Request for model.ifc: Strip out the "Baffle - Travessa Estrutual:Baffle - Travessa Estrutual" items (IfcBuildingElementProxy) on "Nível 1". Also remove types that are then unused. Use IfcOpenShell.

First a look at what the model holds.

```python
import ifcopenshell
import ifcopenshell.util.element

model = ifcopenshell.open("model.ifc")
print(model.schema)
storey = next(s for s in model.by_type("IfcBuildingStorey") if s.Name == "Nível 1")
proxies = [e for e in ifcopenshell.util.element.get_decomposition(storey) if e.is_a("IfcBuildingElementProxy")]
seen = {}
for e in proxies:
    element_type = ifcopenshell.util.element.get_type(e)
    name = element_type.Name if element_type not in (None, e) else None
    seen[name] = seen.get(name, 0) + 1
for name, count in sorted(seen.items(), key=str):
    print(count, "x", name)
```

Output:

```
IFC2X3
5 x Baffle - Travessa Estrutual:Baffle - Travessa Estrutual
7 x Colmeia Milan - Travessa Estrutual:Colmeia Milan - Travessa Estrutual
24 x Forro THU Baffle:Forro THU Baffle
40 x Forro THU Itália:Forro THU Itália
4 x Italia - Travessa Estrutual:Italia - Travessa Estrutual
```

```python
import ifcopenshell
import ifcopenshell.api.root
import ifcopenshell.util.element

model = ifcopenshell.open("model.ifc")

storey = next(s for s in model.by_type("IfcBuildingStorey") if s.Name == "Nível 1")
proxies = [e for e in ifcopenshell.util.element.get_decomposition(storey) if e.is_a("IfcBuildingElementProxy")]
targets = [e for e in proxies if (t := ifcopenshell.util.element.get_type(e)) not in (None, e) and t.Name == "Baffle - Travessa Estrutual:Baffle - Travessa Estrutual"]
types = {ifcopenshell.util.element.get_type(e) for e in targets} - {None, *targets}

for e in targets:
    ifcopenshell.api.root.remove_product(model, product=e)
print(len(targets), "removed")

unused = [t for t in types if not ifcopenshell.util.element.get_types(t)]
for t in unused:
    ifcopenshell.api.root.remove_product(model, product=t)
print(len(unused), "unused types removed")

model.write("model_edited.ifc")
```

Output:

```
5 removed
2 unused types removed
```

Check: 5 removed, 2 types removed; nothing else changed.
